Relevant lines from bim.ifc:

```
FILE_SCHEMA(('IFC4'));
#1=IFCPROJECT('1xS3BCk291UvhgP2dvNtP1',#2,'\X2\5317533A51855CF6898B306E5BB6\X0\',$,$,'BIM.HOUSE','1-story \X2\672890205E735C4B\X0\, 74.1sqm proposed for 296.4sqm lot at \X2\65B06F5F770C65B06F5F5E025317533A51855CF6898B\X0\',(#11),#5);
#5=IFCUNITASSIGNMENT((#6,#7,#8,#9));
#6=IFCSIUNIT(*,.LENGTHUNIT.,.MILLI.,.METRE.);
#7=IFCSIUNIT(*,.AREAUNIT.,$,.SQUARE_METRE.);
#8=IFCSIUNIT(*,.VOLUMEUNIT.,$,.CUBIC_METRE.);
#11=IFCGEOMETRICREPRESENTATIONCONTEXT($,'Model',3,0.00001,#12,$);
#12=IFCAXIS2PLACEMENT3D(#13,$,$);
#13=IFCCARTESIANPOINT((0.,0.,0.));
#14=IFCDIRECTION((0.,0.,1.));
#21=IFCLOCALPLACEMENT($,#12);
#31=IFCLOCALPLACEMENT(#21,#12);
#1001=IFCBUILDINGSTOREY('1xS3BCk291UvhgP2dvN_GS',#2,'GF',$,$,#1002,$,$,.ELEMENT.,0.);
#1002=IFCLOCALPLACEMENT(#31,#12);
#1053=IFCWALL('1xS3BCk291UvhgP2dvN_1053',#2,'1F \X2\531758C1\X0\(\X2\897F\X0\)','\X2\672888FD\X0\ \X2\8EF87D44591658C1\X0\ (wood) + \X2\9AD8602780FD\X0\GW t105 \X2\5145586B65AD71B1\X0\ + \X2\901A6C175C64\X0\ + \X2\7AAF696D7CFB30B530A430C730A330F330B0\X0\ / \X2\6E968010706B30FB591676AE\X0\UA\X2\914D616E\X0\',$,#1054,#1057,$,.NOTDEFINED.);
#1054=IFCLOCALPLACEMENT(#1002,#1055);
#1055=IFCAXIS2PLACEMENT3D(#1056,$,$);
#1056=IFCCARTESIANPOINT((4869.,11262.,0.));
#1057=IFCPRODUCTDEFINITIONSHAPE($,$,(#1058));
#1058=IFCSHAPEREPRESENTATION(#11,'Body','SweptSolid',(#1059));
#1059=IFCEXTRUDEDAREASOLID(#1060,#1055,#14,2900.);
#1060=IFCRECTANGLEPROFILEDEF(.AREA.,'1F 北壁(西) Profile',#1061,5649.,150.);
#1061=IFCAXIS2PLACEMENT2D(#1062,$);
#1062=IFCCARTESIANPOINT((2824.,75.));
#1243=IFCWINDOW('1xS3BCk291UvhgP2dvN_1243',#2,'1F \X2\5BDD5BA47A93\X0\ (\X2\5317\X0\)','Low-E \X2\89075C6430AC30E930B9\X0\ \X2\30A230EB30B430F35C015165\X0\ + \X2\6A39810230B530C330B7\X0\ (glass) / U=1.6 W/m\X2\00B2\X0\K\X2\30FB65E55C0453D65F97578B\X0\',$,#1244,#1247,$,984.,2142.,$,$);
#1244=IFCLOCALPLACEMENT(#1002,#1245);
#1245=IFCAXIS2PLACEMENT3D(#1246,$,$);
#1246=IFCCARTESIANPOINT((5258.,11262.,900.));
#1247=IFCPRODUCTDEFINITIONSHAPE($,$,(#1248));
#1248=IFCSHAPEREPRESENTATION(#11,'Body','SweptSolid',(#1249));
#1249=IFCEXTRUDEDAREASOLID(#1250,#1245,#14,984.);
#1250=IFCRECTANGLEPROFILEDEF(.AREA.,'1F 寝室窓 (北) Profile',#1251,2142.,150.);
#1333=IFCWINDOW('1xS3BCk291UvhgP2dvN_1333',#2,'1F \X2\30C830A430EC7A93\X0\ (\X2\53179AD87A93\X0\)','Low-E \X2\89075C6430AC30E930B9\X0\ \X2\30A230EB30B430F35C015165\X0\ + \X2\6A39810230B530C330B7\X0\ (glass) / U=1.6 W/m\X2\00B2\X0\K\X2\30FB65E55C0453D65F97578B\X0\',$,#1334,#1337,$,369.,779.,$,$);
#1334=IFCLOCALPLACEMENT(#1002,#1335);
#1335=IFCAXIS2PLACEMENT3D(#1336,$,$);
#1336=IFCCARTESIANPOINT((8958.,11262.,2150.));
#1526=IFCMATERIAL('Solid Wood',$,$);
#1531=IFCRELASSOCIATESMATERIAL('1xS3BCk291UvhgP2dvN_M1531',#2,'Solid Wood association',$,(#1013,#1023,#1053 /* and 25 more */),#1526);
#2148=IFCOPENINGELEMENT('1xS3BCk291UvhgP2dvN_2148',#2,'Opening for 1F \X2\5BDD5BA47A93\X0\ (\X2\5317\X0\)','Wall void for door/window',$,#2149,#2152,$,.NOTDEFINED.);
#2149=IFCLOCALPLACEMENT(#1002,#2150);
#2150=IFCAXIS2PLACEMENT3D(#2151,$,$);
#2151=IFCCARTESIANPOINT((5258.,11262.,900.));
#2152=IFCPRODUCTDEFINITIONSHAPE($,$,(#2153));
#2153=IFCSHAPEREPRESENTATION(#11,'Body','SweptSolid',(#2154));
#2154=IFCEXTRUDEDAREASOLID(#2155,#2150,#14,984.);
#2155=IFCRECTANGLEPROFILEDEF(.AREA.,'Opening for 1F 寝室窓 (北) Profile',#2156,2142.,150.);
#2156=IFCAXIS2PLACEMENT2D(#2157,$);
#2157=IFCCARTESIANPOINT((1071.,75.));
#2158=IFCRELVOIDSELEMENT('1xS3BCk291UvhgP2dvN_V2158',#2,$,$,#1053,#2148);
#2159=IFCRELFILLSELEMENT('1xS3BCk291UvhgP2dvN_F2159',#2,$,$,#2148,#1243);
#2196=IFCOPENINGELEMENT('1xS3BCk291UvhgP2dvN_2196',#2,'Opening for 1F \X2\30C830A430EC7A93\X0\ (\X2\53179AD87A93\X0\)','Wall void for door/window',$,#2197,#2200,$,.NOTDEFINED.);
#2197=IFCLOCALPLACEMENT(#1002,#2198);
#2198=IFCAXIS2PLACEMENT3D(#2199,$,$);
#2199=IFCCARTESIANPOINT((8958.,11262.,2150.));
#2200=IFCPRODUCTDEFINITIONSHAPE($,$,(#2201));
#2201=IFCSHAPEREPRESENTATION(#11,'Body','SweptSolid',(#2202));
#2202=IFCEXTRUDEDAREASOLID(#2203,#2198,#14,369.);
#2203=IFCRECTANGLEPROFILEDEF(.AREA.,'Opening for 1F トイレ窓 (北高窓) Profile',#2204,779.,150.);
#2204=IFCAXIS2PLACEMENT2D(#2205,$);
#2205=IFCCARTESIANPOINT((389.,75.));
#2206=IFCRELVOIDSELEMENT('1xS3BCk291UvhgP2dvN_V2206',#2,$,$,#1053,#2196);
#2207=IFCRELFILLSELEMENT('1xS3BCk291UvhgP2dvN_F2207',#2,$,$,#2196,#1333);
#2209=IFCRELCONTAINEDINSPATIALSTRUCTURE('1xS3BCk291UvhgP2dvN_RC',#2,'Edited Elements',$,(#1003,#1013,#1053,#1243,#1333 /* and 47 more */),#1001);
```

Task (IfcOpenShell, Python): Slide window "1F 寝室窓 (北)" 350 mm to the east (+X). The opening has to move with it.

```python
import ifcopenshell
import ifcopenshell.api.geometry
import ifcopenshell.util.placement
import ifcopenshell.util.unit

model = ifcopenshell.open("bim.ifc")
unit_scale = ifcopenshell.util.unit.calculate_unit_scale(model)

window = model.by_guid("1xS3BCk291UvhgP2dvN_1243")
opening = window.FillsVoids[0].RelatingOpeningElement
wall = opening.VoidsElements[0].RelatingBuildingElement

wall_matrix = ifcopenshell.util.placement.get_local_placement(wall.ObjectPlacement)
shift = wall_matrix[:3, 0] * 0.35 / unit_scale
before = ifcopenshell.util.placement.get_local_placement(window.ObjectPlacement)[:3, 3].copy()

# The window is not placed relative to its opening, so move both.
for product in (opening, window):
    matrix = ifcopenshell.util.placement.get_local_placement(product.ObjectPlacement)
    matrix[:3, 3] += shift
    ifcopenshell.api.geometry.edit_object_placement(model, product=product, matrix=matrix, is_si=False)

after = ifcopenshell.util.placement.get_local_placement(window.ObjectPlacement)[:3, 3]
print("window moved by", (after - before).round(3) + 0.0)

model.write("bim_edited.ifc")
```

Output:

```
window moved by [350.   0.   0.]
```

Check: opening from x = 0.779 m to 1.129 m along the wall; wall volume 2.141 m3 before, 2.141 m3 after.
